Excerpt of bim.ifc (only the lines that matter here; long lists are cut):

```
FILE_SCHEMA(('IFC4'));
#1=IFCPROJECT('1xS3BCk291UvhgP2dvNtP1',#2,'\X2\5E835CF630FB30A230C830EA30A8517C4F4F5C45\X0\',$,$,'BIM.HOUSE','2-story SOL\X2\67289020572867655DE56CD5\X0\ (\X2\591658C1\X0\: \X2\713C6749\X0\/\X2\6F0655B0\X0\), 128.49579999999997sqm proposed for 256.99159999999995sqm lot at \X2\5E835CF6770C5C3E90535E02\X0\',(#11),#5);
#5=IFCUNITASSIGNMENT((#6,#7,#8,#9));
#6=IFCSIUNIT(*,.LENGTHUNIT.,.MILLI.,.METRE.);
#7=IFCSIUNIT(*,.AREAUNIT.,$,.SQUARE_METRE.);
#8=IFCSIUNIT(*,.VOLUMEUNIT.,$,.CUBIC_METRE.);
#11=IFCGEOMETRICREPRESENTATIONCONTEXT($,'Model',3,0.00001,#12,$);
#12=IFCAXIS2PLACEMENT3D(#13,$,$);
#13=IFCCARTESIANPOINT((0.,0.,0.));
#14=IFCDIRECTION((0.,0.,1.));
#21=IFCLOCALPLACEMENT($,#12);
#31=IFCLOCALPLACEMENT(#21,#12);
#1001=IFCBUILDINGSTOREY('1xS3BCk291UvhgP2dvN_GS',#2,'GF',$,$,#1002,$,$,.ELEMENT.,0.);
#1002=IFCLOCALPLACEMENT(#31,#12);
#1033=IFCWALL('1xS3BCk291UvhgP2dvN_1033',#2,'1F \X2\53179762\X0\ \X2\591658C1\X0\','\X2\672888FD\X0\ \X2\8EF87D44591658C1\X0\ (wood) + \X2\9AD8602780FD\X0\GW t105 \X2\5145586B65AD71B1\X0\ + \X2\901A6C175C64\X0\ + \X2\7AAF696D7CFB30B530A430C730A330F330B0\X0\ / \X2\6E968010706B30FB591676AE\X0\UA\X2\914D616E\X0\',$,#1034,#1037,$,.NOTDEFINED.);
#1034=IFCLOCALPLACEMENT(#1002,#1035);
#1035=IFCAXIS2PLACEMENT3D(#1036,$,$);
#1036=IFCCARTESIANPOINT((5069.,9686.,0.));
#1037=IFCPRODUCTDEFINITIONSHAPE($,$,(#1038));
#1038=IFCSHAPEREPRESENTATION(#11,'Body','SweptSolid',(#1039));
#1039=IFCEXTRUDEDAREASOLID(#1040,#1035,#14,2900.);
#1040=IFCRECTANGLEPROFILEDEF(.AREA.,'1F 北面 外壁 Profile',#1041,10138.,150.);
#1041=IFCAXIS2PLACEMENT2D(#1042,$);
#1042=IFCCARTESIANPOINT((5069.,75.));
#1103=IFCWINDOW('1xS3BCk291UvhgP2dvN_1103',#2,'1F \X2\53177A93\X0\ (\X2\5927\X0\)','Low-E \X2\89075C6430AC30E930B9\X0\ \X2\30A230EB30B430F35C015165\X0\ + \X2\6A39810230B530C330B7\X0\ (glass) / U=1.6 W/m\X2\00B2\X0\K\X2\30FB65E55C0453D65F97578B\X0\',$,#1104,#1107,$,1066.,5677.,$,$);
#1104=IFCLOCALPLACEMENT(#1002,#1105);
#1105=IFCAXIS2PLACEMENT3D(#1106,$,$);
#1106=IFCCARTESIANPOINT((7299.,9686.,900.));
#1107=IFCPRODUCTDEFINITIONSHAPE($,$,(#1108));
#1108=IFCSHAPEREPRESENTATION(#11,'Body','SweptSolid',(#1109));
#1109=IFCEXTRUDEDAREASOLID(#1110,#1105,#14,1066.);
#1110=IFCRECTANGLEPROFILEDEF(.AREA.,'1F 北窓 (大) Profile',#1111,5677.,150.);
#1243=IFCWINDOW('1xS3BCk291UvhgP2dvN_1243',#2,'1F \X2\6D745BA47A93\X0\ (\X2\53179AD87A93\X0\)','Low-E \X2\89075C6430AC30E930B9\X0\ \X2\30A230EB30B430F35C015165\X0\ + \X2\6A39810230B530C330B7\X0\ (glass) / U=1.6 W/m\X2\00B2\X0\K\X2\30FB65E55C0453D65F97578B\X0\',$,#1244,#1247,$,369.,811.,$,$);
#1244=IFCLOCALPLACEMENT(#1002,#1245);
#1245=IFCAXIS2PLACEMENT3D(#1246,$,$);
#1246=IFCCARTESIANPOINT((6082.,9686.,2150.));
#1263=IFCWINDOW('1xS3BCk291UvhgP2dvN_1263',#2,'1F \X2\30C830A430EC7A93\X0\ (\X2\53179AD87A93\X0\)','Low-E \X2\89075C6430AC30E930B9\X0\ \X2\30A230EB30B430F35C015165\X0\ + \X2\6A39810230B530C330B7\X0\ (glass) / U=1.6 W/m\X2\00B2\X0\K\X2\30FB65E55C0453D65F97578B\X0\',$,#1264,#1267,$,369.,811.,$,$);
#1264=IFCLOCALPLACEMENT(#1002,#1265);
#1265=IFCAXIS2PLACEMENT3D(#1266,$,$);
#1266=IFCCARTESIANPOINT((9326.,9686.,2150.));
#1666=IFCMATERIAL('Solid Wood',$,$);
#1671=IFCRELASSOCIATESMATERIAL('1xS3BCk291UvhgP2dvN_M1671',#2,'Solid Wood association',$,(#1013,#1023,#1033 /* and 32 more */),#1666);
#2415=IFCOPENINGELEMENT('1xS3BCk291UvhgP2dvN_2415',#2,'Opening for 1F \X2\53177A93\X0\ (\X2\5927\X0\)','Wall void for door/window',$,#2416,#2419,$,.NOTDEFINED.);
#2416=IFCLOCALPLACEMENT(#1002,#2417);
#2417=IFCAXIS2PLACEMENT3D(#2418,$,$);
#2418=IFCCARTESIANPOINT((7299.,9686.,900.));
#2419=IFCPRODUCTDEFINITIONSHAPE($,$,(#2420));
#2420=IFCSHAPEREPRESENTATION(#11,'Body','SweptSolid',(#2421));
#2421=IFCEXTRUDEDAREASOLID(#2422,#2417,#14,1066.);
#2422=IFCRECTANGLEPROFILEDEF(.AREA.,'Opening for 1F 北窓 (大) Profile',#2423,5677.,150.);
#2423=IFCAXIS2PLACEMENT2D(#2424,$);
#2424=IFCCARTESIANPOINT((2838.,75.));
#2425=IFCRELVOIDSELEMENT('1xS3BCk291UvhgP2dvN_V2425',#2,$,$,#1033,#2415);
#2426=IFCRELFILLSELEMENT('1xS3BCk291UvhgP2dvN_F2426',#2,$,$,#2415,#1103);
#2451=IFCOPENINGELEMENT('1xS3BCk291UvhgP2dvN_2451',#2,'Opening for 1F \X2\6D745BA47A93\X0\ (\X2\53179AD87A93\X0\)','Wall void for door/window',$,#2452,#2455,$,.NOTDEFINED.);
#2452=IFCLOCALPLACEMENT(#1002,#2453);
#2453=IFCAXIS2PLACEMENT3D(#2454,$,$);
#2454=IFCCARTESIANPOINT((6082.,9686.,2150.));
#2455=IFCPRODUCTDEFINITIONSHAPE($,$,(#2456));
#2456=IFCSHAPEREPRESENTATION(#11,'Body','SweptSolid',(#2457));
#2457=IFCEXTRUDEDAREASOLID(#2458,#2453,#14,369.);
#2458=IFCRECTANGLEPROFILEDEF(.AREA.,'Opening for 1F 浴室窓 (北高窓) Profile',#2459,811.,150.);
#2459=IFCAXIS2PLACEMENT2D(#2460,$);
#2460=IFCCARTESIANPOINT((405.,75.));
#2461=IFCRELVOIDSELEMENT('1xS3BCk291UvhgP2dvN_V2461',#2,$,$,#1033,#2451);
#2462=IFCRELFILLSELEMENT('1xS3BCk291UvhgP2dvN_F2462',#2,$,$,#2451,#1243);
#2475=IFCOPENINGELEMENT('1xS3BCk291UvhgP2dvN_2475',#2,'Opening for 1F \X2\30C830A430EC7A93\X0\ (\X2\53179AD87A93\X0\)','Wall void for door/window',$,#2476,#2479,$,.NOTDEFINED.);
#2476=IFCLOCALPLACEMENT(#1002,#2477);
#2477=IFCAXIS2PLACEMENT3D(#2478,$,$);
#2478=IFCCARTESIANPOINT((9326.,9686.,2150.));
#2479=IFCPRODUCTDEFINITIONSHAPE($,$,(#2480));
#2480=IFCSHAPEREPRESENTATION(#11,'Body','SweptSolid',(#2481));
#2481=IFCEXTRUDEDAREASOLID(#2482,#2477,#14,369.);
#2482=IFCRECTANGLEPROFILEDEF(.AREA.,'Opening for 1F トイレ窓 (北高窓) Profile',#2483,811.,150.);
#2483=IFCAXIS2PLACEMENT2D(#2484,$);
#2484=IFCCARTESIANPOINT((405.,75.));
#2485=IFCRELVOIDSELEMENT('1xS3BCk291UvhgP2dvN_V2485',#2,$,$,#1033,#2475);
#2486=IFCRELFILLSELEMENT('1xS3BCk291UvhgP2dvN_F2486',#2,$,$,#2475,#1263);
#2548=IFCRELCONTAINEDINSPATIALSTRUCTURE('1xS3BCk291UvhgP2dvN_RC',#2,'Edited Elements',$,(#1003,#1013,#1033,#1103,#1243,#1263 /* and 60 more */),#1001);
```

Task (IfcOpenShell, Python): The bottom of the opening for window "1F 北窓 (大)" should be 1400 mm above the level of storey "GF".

```python
import numpy as np
import ifcopenshell
import ifcopenshell.api.geometry
import ifcopenshell.geom
import ifcopenshell.util.element
import ifcopenshell.util.placement
import ifcopenshell.util.shape
import ifcopenshell.util.unit

model = ifcopenshell.open("bim.ifc")
unit_scale = ifcopenshell.util.unit.calculate_unit_scale(model)

window = model.by_id(1103)
opening = window.FillsVoids[0].RelatingOpeningElement
storey = ifcopenshell.util.element.get_container(window, ifc_class="IfcBuildingStorey")
level = ifcopenshell.util.placement.get_local_placement(storey.ObjectPlacement)[2, 3]

# The opening's origin need not be at the sill, so measure its lowest point.
shape = ifcopenshell.geom.create_shape(ifcopenshell.geom.settings(), opening)
bottom = ifcopenshell.util.shape.get_shape_bottom_elevation(shape, shape.geometry) / unit_scale
dz = level + 1.4 / unit_scale - bottom

shift = np.array([0.0, 0.0, dz])
# The window is not placed relative to its opening, so move both.
for product in (opening, window):
    matrix = ifcopenshell.util.placement.get_local_placement(product.ObjectPlacement)
    matrix[:3, 3] += shift
    ifcopenshell.api.geometry.edit_object_placement(model, product=product, matrix=matrix, is_si=False)

print(f"moved by {dz * unit_scale:+.3f} m")

model.write("bim_updated.ifc")
```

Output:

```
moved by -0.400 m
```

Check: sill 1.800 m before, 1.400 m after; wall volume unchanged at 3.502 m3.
